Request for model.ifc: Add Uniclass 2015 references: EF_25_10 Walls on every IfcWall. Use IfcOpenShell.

First a look at what the model holds.

```python
import ifcopenshell

model = ifcopenshell.open("model.ifc")
print(model.schema)
print("classifications:", [c.Name for c in model.by_type("IfcClassification")])
for ifc_class in ("IfcDoor", "IfcRoof", "IfcStair", "IfcWall", "IfcWindow"):
    print(ifc_class, len(model.by_type(ifc_class)))
```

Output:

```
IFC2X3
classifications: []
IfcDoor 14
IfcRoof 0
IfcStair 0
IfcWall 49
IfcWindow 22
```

```python
import ifcopenshell
import ifcopenshell.api.classification

model = ifcopenshell.open("model.ifc")

# IFC2X3 requires Source and Edition and has no link from the project to the system.
system = model.create_entity("IfcClassification", Source="NBS", Edition="2015", Name="Uniclass 2015")

codes = {
    "IfcWall": ("EF_25_10", "Walls"),
}
for ifc_class, (code, name) in codes.items():
    products = model.by_type(ifc_class)
    ifcopenshell.api.classification.add_reference(
        model, products=products, classification=system, identification=code, name=name
    )
    print(code, len(products))

model.write("model_edited.ifc")
```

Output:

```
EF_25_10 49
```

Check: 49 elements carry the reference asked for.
